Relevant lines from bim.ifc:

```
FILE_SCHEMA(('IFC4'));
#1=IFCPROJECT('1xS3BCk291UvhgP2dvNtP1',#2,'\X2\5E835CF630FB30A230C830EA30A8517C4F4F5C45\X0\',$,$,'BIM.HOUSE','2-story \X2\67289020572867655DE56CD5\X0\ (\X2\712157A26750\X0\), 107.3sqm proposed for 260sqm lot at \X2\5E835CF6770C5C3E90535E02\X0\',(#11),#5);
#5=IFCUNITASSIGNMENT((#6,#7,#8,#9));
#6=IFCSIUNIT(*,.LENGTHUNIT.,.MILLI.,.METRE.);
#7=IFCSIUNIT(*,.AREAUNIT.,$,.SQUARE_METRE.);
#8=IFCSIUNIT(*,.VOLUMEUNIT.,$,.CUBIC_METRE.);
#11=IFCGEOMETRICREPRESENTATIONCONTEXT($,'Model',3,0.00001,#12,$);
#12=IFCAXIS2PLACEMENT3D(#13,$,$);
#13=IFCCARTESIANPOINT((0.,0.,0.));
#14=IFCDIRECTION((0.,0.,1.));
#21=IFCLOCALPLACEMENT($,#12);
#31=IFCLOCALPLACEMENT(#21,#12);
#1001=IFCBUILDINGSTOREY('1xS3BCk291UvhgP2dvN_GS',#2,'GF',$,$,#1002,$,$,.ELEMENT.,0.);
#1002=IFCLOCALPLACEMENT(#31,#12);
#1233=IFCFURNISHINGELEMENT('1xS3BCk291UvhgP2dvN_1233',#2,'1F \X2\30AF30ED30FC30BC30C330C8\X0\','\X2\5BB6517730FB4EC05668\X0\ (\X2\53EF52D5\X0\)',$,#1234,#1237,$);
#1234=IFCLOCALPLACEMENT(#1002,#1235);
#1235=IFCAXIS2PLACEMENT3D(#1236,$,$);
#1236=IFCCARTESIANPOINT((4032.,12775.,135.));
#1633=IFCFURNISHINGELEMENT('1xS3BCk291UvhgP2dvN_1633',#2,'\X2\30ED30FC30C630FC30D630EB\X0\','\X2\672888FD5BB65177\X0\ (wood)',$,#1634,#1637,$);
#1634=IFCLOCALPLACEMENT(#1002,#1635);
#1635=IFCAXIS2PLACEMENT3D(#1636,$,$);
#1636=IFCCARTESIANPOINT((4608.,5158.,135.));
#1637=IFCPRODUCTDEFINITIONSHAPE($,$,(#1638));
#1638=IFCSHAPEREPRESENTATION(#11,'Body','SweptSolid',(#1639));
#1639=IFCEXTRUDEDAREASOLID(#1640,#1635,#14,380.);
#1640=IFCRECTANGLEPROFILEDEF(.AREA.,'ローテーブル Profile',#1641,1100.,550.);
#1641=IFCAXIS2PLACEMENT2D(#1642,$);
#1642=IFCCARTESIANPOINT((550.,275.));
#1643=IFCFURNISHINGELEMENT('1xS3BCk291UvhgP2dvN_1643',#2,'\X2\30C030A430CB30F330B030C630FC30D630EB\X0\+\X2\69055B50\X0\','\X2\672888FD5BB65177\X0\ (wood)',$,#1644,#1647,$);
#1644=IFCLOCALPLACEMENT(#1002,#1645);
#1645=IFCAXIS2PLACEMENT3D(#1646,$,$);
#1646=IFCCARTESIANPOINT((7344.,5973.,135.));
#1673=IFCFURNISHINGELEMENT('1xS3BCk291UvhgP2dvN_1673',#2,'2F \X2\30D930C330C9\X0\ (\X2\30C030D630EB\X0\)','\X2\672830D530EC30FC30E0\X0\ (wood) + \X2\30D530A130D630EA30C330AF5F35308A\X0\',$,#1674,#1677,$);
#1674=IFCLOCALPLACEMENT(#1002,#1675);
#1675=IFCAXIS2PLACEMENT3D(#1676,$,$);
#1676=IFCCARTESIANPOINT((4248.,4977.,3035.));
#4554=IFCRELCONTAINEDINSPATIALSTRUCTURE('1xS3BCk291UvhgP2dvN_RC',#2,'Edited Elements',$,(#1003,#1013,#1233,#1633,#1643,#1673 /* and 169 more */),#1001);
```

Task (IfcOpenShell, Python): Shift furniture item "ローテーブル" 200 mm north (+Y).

```python
import ifcopenshell
import ifcopenshell.api.geometry
import ifcopenshell.util.placement
import ifcopenshell.util.unit

model = ifcopenshell.open("bim.ifc")
unit_scale = ifcopenshell.util.unit.calculate_unit_scale(model)

item = model.by_id(1633)
matrix = ifcopenshell.util.placement.get_local_placement(item.ObjectPlacement)
matrix[1, 3] += 0.2 / unit_scale
ifcopenshell.api.geometry.edit_object_placement(model, product=item, matrix=matrix, is_si=False)

print(ifcopenshell.util.placement.get_local_placement(item.ObjectPlacement).round(3) + 0.0)

model.write("bim_v2.ifc")
```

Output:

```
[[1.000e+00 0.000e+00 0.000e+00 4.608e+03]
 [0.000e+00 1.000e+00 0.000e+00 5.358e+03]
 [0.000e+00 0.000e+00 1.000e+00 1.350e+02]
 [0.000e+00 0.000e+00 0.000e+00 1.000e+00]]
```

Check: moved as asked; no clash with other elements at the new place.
